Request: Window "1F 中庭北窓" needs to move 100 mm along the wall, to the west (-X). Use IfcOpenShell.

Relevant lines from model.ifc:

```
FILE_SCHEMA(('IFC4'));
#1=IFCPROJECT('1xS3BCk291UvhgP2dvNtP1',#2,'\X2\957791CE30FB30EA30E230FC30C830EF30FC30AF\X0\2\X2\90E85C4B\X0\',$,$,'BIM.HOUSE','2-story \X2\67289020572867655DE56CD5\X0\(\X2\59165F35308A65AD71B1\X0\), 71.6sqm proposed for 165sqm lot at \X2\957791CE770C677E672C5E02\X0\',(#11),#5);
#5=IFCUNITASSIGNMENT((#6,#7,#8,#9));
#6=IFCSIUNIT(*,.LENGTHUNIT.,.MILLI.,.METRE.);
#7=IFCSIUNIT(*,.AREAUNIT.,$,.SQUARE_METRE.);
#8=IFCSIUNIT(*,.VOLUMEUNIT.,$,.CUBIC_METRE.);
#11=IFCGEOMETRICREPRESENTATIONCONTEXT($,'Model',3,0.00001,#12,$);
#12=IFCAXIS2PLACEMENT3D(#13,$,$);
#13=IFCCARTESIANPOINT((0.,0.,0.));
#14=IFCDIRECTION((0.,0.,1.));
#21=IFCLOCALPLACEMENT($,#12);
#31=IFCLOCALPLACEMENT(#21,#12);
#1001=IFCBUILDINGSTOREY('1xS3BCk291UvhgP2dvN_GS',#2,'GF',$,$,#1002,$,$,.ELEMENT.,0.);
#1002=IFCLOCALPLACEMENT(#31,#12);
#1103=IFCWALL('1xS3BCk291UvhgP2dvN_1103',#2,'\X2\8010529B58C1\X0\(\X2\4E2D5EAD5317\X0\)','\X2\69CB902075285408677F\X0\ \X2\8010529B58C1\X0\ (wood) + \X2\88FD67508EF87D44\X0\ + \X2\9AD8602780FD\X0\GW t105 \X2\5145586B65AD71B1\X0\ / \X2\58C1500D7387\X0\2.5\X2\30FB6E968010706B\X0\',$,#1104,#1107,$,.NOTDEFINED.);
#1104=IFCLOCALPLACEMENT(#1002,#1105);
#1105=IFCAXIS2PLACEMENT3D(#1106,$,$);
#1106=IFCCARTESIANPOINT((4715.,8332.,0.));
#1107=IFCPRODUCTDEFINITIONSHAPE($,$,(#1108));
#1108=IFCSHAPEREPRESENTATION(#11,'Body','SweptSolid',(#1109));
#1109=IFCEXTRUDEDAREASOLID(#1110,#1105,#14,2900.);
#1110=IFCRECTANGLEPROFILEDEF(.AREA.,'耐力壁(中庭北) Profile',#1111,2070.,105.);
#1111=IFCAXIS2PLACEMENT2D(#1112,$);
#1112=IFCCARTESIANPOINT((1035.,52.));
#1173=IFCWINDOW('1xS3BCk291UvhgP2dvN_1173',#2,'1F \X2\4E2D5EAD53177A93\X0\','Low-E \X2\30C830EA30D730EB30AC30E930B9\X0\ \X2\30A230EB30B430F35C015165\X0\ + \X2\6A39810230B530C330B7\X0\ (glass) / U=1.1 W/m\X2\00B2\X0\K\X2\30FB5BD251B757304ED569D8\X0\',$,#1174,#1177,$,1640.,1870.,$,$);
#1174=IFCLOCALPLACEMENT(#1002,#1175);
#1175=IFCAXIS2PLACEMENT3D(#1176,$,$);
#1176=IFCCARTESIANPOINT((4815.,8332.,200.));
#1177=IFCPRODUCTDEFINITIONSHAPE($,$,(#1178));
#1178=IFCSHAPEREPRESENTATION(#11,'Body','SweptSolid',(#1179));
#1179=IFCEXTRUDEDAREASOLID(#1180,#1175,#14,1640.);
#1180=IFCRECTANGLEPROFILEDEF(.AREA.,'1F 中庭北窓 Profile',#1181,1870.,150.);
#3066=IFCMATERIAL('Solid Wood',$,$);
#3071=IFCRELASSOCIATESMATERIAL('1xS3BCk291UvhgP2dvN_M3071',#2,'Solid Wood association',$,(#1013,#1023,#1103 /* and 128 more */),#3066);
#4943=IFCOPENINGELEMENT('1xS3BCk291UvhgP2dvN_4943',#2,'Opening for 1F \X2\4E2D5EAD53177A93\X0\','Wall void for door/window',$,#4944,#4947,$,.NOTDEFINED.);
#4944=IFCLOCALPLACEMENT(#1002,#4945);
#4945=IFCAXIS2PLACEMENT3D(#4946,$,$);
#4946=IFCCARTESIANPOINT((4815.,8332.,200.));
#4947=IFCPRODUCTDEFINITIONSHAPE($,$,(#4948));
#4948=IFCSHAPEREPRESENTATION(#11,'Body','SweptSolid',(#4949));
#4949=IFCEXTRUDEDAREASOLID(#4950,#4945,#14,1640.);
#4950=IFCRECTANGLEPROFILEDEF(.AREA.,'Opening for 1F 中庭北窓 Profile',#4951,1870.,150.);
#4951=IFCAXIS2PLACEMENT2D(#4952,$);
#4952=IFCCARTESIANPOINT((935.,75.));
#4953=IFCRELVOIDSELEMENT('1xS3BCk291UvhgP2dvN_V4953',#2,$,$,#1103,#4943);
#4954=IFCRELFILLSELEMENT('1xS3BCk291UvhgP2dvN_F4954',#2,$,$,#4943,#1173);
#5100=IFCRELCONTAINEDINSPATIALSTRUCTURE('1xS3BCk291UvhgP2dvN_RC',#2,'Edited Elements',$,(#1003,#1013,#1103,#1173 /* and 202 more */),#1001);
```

```python
import ifcopenshell
import ifcopenshell.api.geometry
import ifcopenshell.util.placement
import ifcopenshell.util.unit

model = ifcopenshell.open("model.ifc")
unit_scale = ifcopenshell.util.unit.calculate_unit_scale(model)

window = model.by_guid("1xS3BCk291UvhgP2dvN_1173")
opening = window.FillsVoids[0].RelatingOpeningElement
wall = opening.VoidsElements[0].RelatingBuildingElement

wall_matrix = ifcopenshell.util.placement.get_local_placement(wall.ObjectPlacement)
shift = wall_matrix[:3, 0] * -0.1 / unit_scale
before = ifcopenshell.util.placement.get_local_placement(window.ObjectPlacement)[:3, 3].copy()

# The window is not placed relative to its opening, so move both.
for product in (opening, window):
    matrix = ifcopenshell.util.placement.get_local_placement(product.ObjectPlacement)
    matrix[:3, 3] += shift
    ifcopenshell.api.geometry.edit_object_placement(model, product=product, matrix=matrix, is_si=False)

after = ifcopenshell.util.placement.get_local_placement(window.ObjectPlacement)[:3, 3]
print("window moved by", (after - before).round(3) + 0.0)

model.write("model_rev.ifc")
```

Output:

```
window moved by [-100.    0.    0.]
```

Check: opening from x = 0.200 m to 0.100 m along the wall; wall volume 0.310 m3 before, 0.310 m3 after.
